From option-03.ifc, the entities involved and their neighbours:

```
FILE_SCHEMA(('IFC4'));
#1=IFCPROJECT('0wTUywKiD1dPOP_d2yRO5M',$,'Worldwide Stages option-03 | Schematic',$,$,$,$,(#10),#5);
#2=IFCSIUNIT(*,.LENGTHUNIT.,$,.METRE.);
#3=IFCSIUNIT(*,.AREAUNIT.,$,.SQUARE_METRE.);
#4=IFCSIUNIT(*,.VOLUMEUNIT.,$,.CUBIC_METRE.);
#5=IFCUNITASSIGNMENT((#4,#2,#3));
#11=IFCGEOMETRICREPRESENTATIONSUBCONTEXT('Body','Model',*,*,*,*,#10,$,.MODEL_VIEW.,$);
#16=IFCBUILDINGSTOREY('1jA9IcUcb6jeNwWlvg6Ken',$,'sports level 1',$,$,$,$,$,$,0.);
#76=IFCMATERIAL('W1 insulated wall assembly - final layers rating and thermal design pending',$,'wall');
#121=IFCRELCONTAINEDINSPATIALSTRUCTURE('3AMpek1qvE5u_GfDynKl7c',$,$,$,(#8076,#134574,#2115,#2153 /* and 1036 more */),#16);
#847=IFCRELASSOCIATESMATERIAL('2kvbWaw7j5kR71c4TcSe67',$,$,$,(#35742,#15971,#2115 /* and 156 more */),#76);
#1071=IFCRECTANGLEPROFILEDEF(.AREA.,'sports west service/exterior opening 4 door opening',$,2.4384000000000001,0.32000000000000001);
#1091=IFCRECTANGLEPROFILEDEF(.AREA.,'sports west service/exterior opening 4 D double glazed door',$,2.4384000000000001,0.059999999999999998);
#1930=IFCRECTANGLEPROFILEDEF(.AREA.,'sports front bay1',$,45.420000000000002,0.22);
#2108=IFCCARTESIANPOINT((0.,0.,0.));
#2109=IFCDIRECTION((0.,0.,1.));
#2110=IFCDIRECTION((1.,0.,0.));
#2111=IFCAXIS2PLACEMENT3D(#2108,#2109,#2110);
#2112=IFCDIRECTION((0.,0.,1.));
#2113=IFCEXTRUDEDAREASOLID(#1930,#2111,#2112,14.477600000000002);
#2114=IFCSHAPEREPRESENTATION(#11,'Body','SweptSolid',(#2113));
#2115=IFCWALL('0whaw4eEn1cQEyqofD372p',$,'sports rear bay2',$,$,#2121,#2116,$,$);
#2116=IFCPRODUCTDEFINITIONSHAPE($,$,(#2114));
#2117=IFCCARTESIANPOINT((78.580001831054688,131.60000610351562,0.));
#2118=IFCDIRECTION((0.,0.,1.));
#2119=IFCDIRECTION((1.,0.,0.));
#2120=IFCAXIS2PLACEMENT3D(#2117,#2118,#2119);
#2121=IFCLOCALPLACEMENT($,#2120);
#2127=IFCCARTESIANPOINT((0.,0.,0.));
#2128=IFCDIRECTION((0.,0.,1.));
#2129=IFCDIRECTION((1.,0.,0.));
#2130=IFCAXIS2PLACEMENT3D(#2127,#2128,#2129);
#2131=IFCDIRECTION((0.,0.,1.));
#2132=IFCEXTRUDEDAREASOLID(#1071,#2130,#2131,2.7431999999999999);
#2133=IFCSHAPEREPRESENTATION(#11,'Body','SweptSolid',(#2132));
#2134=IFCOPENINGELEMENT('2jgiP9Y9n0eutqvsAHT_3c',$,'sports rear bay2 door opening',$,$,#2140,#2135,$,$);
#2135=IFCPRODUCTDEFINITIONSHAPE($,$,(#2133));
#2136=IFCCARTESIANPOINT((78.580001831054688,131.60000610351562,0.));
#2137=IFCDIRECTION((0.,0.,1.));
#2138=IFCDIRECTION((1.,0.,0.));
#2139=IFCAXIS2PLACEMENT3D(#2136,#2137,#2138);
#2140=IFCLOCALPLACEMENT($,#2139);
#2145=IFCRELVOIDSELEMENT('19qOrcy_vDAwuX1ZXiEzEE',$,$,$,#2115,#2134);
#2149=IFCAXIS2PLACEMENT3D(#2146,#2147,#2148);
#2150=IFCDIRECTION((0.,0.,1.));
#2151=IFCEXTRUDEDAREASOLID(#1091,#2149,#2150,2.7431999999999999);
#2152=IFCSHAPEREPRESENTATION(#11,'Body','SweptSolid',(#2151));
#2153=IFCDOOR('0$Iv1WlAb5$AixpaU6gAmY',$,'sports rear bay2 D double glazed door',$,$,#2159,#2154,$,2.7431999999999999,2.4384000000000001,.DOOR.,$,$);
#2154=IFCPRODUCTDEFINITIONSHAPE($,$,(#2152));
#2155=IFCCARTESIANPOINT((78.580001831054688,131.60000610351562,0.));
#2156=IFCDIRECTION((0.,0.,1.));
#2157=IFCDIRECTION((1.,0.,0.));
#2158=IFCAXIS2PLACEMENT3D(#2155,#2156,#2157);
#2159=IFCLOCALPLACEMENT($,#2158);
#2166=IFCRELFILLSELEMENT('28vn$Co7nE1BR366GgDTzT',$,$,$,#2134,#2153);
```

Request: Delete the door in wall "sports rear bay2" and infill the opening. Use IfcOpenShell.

```python
import ifcopenshell
import ifcopenshell.api.feature
import ifcopenshell.api.root
import ifcopenshell.geom
import ifcopenshell.util.shape

model = ifcopenshell.open("option-03.ifc")
settings = ifcopenshell.geom.settings()


def volume(element):
    """Net volume in cubic metres, openings subtracted."""
    shape = ifcopenshell.geom.create_shape(settings, element)
    return ifcopenshell.util.shape.get_volume(shape.geometry)


door = model.by_guid("0$Iv1WlAb5$AixpaU6gAmY")
opening = door.FillsVoids[0].RelatingOpeningElement
wall = opening.VoidsElements[0].RelatingBuildingElement
before = volume(wall)

ifcopenshell.api.root.remove_product(model, product=door)
ifcopenshell.api.feature.remove_feature(model, feature=opening)

after = volume(wall)

print(f"wall volume {before:.3f} -> {after:.3f} m3")

model.write("option-03_v2.ifc")
```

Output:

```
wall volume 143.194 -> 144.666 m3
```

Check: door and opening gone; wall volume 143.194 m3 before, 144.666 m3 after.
